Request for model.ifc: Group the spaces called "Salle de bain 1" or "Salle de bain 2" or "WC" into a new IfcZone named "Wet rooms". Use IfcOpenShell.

First a look at what the model holds.

```python
import ifcopenshell

model = ifcopenshell.open("model.ifc")
print(model.schema)
seen = {}
for space in model.by_type("IfcSpace"):
    seen[space.LongName] = seen.get(space.LongName, 0) + 1
for name, count in sorted(seen.items(), key=str):
    print(count, "x", name)
print("zones:", [z.Name for z in model.by_type("IfcZone")][:20])
```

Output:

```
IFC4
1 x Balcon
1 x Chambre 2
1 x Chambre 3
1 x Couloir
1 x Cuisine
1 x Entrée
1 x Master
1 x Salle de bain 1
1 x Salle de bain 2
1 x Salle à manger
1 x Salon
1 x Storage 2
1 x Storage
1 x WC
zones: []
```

```python
import ifcopenshell
import ifcopenshell.api.group
import ifcopenshell.api.root

model = ifcopenshell.open("model.ifc")

names = {"Salle de bain 1", "Salle de bain 2", "WC"}
spaces = [s for s in model.by_type("IfcSpace") if s.LongName in names]

zone = ifcopenshell.api.root.create_entity(model, ifc_class="IfcZone", name="Wet rooms")
ifcopenshell.api.group.assign_group(model, products=spaces, group=zone)
print(len(spaces), "spaces in", zone.Name)

model.write("model_edited.ifc")
```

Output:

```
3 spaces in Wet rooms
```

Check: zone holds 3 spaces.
